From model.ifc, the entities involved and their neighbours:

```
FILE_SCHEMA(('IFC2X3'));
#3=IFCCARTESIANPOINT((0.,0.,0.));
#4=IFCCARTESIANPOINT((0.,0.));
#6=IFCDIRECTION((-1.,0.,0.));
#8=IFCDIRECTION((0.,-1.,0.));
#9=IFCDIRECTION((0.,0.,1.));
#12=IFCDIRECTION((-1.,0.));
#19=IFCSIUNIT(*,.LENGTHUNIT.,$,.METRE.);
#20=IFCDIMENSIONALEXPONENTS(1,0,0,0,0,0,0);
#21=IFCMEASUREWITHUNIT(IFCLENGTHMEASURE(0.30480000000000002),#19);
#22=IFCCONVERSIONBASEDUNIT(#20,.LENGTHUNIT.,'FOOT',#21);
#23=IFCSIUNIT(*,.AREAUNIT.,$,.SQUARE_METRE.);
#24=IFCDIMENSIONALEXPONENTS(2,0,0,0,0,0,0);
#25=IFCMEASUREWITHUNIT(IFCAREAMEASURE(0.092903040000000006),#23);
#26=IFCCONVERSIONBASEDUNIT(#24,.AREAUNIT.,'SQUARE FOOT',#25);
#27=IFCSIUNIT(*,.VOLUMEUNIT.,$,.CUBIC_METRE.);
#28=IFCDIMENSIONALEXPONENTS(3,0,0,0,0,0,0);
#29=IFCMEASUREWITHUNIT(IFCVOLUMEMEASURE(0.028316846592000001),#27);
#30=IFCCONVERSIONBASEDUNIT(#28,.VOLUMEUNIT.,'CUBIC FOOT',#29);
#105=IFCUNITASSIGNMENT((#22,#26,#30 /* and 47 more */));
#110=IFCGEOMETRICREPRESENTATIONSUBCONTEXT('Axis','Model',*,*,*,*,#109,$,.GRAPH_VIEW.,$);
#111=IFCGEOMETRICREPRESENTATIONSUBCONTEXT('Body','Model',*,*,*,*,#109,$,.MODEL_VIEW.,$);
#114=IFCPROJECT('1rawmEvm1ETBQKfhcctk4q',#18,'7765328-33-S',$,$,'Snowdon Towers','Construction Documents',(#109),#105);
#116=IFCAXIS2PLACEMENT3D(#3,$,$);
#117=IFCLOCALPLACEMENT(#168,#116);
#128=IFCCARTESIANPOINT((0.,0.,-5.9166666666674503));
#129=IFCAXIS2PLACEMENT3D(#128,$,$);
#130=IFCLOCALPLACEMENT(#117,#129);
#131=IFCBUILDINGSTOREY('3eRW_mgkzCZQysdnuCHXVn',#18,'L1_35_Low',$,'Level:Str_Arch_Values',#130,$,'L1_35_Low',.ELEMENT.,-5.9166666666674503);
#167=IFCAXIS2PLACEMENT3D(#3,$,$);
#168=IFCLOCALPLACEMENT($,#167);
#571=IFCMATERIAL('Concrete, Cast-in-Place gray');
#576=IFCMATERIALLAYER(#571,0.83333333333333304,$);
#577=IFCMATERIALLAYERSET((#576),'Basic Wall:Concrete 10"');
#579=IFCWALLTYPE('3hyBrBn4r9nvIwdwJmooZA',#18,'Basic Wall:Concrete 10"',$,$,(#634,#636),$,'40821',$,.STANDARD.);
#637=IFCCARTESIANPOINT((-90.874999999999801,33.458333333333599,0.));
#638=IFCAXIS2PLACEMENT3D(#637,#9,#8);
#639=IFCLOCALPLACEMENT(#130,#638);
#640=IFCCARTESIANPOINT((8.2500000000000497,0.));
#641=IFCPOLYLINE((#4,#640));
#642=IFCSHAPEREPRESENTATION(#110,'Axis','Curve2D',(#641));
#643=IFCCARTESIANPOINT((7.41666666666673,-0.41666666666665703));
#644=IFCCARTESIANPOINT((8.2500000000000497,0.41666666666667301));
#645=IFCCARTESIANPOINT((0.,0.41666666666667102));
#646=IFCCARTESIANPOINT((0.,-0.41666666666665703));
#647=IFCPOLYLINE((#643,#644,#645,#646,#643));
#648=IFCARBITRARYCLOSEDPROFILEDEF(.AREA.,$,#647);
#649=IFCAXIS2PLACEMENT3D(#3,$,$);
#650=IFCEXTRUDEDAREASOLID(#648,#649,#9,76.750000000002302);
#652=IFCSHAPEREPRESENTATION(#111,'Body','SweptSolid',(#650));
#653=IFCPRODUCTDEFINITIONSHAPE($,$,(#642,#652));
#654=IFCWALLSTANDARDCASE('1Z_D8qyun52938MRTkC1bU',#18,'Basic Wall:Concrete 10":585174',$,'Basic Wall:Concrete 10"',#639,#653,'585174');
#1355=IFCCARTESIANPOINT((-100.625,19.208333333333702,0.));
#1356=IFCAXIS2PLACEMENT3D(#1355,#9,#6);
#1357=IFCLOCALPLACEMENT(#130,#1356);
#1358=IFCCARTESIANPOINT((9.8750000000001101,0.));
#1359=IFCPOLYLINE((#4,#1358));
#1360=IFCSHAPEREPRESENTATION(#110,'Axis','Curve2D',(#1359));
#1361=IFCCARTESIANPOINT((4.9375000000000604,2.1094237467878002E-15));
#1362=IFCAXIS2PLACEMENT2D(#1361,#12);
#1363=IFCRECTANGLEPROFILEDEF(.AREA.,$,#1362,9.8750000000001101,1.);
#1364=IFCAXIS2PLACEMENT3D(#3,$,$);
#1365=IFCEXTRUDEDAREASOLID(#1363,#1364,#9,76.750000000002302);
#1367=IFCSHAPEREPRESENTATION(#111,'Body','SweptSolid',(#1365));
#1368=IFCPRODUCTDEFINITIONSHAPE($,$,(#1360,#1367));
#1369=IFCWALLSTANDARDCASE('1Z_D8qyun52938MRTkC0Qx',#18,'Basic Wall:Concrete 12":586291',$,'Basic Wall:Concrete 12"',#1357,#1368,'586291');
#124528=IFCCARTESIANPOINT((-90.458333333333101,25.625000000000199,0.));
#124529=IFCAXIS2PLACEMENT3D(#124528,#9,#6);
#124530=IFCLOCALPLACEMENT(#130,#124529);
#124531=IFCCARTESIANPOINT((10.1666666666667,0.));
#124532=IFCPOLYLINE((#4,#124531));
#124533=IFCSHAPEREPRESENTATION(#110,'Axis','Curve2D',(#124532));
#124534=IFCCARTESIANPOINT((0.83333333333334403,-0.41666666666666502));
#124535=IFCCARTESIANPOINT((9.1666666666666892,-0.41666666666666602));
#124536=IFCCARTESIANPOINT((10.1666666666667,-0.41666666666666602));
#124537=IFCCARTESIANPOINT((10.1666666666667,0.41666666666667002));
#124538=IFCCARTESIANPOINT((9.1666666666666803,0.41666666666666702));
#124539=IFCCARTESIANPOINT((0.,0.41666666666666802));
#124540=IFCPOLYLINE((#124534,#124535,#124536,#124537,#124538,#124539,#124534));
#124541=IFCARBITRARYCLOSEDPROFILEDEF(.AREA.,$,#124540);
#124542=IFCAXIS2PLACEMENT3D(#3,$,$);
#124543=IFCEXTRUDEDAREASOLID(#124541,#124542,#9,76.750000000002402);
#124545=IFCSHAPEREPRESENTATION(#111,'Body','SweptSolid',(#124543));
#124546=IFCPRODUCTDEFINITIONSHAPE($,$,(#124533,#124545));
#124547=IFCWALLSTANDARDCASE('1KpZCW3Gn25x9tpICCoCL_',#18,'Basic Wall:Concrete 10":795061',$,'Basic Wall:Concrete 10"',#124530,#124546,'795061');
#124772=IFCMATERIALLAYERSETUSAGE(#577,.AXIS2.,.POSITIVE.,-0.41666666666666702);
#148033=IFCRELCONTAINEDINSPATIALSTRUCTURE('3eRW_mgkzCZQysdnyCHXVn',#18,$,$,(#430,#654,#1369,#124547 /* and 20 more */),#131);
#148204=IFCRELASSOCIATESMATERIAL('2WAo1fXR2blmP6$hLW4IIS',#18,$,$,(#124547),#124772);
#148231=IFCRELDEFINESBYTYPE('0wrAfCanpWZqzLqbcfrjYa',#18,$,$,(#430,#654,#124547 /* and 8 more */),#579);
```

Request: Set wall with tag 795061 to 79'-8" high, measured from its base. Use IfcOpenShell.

```python
import ifcopenshell
import ifcopenshell.geom
import ifcopenshell.util.representation
import ifcopenshell.util.shape
import ifcopenshell.util.unit

model = ifcopenshell.open("model.ifc")
unit_scale = ifcopenshell.util.unit.calculate_unit_scale(model)
settings = ifcopenshell.geom.settings()


def volume(element):
    """Net volume in cubic metres, openings subtracted."""
    shape = ifcopenshell.geom.create_shape(settings, element)
    return ifcopenshell.util.shape.get_volume(shape.geometry)


wall = model.by_guid("1KpZCW3Gn25x9tpICCoCL_")
before = volume(wall)

body = ifcopenshell.util.representation.get_representation(wall, "Model", "Body")
solid = body.Items[0]
old_height = solid.Depth
solid.Depth = 956 * 0.0254 / unit_scale
after = volume(wall)

print(f"height {old_height:g} -> {solid.Depth:g}, volume {before:.3f} -> {after:.3f} m3")

model.write("model_updated.ifc")
```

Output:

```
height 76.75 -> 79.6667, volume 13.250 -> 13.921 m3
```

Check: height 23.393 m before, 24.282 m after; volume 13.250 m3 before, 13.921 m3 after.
